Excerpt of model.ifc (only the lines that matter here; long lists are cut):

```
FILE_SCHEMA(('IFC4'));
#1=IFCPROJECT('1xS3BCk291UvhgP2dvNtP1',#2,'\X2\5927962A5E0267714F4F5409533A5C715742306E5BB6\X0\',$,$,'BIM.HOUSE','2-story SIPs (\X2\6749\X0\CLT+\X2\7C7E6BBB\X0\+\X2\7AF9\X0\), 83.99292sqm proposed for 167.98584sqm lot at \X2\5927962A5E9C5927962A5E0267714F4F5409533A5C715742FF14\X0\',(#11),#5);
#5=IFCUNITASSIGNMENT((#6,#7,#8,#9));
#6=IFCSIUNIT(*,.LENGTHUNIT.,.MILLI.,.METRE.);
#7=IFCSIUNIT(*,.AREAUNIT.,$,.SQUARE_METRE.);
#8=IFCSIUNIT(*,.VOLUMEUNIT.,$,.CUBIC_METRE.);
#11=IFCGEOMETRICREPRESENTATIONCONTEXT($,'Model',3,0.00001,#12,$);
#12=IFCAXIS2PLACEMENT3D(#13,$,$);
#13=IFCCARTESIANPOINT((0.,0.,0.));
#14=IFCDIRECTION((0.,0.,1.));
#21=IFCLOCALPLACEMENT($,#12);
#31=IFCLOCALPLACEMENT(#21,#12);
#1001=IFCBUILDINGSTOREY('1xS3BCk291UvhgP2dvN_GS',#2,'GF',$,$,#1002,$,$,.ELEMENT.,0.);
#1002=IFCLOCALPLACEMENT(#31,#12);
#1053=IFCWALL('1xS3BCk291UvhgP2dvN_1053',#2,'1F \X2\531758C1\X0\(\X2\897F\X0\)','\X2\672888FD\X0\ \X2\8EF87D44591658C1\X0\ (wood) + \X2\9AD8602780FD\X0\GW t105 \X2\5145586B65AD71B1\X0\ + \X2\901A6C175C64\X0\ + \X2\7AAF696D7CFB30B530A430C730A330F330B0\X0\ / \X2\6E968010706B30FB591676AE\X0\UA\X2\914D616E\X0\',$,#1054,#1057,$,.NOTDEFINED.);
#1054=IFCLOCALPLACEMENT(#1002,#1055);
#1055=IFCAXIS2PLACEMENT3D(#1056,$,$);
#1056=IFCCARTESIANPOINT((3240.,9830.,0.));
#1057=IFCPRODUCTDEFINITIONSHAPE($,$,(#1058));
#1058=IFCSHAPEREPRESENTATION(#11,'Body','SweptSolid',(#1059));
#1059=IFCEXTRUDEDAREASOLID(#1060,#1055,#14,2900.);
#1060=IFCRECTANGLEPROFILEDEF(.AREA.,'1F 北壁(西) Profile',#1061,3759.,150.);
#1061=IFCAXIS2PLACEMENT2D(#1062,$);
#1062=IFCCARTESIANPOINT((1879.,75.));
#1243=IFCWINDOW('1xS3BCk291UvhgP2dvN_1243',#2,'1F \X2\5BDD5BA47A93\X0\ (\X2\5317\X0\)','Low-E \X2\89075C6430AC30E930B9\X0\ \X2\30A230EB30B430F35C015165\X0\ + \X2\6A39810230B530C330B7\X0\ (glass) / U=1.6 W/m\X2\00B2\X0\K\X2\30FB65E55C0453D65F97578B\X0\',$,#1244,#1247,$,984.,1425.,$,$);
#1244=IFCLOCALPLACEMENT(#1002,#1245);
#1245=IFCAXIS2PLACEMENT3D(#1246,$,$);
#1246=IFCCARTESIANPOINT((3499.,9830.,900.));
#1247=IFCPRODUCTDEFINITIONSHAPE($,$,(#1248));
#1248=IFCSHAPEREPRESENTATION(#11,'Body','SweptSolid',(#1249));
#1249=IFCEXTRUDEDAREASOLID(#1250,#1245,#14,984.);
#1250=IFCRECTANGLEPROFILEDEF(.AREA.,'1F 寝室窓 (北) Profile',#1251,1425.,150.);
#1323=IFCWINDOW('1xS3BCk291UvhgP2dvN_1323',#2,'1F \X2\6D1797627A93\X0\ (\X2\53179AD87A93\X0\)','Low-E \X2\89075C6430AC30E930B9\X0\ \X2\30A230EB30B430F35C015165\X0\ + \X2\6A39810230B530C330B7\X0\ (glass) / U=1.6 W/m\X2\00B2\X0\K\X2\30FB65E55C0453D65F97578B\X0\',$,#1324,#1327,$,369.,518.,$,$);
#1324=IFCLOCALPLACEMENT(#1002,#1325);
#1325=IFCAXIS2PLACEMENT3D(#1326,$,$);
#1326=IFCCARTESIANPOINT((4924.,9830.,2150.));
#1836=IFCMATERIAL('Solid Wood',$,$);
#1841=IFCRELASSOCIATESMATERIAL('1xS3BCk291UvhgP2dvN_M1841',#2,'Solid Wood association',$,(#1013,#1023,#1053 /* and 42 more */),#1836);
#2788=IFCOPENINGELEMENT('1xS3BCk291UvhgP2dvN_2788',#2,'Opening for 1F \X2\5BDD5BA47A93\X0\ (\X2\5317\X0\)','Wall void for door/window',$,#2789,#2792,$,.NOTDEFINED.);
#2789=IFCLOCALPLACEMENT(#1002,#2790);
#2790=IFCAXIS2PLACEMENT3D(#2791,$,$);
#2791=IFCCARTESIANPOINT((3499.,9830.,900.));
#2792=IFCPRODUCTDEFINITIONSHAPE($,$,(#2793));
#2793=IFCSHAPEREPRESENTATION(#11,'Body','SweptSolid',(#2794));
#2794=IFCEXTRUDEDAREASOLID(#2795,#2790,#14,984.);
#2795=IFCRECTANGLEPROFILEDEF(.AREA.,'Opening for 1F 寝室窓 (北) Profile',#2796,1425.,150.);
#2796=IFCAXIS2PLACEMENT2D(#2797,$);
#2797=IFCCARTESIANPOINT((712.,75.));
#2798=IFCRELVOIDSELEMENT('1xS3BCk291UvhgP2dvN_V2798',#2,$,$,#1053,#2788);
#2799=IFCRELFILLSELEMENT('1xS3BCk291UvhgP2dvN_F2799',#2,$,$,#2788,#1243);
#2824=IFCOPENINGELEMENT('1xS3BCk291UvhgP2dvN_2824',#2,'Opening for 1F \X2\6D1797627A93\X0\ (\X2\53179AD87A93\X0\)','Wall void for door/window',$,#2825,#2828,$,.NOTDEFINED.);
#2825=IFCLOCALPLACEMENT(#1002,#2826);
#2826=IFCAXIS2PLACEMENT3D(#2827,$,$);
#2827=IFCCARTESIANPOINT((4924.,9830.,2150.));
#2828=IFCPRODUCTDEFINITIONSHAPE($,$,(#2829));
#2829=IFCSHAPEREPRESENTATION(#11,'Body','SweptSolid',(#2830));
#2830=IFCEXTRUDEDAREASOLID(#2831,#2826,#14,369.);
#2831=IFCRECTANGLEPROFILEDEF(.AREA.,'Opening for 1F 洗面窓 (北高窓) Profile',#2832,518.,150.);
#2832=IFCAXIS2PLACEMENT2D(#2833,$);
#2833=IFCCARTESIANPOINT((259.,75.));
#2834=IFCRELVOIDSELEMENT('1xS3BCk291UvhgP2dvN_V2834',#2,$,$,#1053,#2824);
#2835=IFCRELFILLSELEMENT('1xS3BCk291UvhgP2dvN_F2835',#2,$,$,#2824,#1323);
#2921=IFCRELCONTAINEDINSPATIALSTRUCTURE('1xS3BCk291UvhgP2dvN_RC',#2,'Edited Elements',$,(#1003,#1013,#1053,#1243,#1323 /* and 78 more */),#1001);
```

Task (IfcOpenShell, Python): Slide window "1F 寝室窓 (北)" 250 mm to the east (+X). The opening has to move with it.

```python
import ifcopenshell
import ifcopenshell.api.geometry
import ifcopenshell.util.placement

model = ifcopenshell.open("model.ifc")

window = model.by_guid("1xS3BCk291UvhgP2dvN_1243")
opening = window.FillsVoids[0].RelatingOpeningElement
wall = opening.VoidsElements[0].RelatingBuildingElement

wall_matrix = ifcopenshell.util.placement.get_local_placement(wall.ObjectPlacement)
shift = wall_matrix[:3, 0] * 250.0
before = ifcopenshell.util.placement.get_local_placement(window.ObjectPlacement)[:3, 3].copy()

# The window is not placed relative to its opening, so move both.
for product in (opening, window):
    matrix = ifcopenshell.util.placement.get_local_placement(product.ObjectPlacement)
    matrix[:3, 3] += shift
    ifcopenshell.api.geometry.edit_object_placement(model, product=product, matrix=matrix, is_si=False)

after = ifcopenshell.util.placement.get_local_placement(window.ObjectPlacement)[:3, 3]
print("window moved by", (after - before).round(3) + 0.0)

model.write("model_edited.ifc")
```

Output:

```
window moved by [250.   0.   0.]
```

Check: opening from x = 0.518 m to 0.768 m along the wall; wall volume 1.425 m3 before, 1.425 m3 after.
